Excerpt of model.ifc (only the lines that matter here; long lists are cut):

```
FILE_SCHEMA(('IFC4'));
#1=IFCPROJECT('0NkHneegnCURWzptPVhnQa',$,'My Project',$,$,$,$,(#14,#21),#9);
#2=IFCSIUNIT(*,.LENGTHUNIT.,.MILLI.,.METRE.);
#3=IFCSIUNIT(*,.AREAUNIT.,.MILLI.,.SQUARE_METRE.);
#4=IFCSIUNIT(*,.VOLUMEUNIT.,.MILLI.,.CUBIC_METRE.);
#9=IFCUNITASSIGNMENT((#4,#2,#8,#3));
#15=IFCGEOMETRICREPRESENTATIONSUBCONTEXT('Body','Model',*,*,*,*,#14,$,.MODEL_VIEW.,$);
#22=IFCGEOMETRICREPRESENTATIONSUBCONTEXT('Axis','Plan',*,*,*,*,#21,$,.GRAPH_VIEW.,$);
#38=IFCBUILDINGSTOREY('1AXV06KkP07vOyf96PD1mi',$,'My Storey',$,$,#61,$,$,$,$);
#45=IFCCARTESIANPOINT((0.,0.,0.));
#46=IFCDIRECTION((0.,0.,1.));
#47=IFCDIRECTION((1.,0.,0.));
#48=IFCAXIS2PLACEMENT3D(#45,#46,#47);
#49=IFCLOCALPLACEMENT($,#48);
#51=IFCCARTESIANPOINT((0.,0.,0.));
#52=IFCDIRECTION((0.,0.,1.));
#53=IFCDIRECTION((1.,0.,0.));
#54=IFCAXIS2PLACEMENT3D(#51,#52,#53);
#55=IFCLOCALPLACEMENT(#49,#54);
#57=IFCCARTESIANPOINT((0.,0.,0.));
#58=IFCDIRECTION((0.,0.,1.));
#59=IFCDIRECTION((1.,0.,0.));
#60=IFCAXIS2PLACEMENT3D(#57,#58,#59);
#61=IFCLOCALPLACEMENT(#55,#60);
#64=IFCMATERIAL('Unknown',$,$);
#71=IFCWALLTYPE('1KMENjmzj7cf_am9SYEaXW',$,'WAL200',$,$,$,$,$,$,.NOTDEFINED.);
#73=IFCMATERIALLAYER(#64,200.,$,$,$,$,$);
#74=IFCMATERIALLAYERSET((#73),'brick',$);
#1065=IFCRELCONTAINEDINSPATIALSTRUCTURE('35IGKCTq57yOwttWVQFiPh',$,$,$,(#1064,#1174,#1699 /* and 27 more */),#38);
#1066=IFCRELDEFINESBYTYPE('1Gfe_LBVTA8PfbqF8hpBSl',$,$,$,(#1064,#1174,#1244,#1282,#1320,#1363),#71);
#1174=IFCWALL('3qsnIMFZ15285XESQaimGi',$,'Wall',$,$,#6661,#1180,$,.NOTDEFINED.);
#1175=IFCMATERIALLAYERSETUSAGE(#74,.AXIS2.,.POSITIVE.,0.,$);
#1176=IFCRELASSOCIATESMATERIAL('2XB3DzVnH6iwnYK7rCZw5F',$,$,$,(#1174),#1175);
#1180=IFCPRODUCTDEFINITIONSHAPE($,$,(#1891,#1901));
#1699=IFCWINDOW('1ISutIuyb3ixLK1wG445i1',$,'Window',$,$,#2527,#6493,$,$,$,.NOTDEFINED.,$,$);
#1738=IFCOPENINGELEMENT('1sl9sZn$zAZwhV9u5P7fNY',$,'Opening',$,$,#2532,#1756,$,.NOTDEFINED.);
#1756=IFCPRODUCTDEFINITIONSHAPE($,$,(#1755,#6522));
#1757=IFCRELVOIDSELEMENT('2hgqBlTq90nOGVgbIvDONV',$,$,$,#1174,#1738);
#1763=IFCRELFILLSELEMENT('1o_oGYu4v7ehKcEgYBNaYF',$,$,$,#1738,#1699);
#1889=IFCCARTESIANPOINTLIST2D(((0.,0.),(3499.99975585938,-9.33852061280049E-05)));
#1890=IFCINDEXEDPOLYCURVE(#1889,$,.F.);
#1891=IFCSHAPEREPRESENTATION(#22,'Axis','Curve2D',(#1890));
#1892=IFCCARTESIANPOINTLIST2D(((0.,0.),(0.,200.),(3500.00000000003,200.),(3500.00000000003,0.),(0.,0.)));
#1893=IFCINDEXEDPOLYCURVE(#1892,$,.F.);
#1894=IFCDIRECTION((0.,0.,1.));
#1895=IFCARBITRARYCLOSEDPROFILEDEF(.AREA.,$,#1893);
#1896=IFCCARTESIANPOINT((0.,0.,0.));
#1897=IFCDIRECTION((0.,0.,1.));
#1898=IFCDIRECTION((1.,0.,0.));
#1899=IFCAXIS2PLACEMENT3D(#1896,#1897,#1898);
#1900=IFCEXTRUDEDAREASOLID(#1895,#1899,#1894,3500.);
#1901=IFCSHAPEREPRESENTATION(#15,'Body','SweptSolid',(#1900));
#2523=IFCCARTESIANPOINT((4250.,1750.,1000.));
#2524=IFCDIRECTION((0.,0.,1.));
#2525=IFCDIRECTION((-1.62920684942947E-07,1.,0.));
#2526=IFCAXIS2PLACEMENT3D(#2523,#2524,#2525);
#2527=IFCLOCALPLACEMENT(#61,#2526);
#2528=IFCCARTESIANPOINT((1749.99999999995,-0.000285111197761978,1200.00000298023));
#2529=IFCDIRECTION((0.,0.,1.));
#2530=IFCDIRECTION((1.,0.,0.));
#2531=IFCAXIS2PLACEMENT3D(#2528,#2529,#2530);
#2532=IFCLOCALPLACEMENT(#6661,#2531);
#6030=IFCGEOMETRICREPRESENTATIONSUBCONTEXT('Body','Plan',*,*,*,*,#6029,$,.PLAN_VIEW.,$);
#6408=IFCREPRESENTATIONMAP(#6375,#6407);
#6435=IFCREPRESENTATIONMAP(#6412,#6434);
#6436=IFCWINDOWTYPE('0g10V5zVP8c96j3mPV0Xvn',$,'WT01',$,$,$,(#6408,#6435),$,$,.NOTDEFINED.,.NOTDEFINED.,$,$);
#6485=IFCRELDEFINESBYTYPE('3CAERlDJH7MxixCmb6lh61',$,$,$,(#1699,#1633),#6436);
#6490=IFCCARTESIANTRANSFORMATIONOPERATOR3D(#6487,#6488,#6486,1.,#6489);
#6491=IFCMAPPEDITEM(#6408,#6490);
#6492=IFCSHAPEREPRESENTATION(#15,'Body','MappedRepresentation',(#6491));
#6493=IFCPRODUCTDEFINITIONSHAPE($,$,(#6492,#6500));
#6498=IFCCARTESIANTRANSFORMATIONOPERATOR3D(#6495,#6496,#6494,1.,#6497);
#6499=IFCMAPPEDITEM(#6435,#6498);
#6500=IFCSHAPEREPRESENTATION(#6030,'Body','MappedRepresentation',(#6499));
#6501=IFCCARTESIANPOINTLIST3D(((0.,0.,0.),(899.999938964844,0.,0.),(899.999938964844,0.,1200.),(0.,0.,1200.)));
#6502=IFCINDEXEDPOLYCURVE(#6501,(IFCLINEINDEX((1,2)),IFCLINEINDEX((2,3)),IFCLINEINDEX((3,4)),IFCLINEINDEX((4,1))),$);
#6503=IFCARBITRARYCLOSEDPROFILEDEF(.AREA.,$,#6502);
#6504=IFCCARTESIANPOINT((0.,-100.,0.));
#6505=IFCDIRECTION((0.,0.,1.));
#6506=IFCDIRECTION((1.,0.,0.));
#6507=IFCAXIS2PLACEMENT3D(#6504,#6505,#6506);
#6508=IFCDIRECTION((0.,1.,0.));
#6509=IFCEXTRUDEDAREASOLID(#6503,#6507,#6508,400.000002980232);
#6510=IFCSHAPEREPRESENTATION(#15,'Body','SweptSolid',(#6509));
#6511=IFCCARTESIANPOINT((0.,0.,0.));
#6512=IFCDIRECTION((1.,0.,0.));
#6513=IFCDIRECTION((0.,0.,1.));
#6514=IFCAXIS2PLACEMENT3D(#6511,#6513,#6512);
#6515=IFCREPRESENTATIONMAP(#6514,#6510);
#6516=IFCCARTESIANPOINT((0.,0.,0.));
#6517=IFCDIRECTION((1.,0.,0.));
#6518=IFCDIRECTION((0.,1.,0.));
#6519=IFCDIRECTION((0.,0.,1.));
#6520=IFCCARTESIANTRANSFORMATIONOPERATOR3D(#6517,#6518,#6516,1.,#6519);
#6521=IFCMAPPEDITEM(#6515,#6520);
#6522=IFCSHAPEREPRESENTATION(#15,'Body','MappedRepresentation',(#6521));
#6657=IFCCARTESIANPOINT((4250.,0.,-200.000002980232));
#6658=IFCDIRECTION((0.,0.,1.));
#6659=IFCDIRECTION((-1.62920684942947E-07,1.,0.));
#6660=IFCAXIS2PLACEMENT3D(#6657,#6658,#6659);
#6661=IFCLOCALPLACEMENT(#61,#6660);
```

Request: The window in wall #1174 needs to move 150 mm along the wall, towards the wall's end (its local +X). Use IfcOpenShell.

```python
import ifcopenshell
import ifcopenshell.api.geometry
import ifcopenshell.util.placement

model = ifcopenshell.open("model.ifc")

window = model.by_id(1699)
opening = window.FillsVoids[0].RelatingOpeningElement
wall = opening.VoidsElements[0].RelatingBuildingElement

wall_matrix = ifcopenshell.util.placement.get_local_placement(wall.ObjectPlacement)
shift = wall_matrix[:3, 0] * 150.0
before = ifcopenshell.util.placement.get_local_placement(window.ObjectPlacement)[:3, 3].copy()

# The window is not placed relative to its opening, so move both.
for product in (opening, window):
    matrix = ifcopenshell.util.placement.get_local_placement(product.ObjectPlacement)
    matrix[:3, 3] += shift
    ifcopenshell.api.geometry.edit_object_placement(model, product=product, matrix=matrix, is_si=False)

after = ifcopenshell.util.placement.get_local_placement(window.ObjectPlacement)[:3, 3]
print("window moved by", (after - before).round(3) + 0.0)

model.write("model_rev.ifc")
```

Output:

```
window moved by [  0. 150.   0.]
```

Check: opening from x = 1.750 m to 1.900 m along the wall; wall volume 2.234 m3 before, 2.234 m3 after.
